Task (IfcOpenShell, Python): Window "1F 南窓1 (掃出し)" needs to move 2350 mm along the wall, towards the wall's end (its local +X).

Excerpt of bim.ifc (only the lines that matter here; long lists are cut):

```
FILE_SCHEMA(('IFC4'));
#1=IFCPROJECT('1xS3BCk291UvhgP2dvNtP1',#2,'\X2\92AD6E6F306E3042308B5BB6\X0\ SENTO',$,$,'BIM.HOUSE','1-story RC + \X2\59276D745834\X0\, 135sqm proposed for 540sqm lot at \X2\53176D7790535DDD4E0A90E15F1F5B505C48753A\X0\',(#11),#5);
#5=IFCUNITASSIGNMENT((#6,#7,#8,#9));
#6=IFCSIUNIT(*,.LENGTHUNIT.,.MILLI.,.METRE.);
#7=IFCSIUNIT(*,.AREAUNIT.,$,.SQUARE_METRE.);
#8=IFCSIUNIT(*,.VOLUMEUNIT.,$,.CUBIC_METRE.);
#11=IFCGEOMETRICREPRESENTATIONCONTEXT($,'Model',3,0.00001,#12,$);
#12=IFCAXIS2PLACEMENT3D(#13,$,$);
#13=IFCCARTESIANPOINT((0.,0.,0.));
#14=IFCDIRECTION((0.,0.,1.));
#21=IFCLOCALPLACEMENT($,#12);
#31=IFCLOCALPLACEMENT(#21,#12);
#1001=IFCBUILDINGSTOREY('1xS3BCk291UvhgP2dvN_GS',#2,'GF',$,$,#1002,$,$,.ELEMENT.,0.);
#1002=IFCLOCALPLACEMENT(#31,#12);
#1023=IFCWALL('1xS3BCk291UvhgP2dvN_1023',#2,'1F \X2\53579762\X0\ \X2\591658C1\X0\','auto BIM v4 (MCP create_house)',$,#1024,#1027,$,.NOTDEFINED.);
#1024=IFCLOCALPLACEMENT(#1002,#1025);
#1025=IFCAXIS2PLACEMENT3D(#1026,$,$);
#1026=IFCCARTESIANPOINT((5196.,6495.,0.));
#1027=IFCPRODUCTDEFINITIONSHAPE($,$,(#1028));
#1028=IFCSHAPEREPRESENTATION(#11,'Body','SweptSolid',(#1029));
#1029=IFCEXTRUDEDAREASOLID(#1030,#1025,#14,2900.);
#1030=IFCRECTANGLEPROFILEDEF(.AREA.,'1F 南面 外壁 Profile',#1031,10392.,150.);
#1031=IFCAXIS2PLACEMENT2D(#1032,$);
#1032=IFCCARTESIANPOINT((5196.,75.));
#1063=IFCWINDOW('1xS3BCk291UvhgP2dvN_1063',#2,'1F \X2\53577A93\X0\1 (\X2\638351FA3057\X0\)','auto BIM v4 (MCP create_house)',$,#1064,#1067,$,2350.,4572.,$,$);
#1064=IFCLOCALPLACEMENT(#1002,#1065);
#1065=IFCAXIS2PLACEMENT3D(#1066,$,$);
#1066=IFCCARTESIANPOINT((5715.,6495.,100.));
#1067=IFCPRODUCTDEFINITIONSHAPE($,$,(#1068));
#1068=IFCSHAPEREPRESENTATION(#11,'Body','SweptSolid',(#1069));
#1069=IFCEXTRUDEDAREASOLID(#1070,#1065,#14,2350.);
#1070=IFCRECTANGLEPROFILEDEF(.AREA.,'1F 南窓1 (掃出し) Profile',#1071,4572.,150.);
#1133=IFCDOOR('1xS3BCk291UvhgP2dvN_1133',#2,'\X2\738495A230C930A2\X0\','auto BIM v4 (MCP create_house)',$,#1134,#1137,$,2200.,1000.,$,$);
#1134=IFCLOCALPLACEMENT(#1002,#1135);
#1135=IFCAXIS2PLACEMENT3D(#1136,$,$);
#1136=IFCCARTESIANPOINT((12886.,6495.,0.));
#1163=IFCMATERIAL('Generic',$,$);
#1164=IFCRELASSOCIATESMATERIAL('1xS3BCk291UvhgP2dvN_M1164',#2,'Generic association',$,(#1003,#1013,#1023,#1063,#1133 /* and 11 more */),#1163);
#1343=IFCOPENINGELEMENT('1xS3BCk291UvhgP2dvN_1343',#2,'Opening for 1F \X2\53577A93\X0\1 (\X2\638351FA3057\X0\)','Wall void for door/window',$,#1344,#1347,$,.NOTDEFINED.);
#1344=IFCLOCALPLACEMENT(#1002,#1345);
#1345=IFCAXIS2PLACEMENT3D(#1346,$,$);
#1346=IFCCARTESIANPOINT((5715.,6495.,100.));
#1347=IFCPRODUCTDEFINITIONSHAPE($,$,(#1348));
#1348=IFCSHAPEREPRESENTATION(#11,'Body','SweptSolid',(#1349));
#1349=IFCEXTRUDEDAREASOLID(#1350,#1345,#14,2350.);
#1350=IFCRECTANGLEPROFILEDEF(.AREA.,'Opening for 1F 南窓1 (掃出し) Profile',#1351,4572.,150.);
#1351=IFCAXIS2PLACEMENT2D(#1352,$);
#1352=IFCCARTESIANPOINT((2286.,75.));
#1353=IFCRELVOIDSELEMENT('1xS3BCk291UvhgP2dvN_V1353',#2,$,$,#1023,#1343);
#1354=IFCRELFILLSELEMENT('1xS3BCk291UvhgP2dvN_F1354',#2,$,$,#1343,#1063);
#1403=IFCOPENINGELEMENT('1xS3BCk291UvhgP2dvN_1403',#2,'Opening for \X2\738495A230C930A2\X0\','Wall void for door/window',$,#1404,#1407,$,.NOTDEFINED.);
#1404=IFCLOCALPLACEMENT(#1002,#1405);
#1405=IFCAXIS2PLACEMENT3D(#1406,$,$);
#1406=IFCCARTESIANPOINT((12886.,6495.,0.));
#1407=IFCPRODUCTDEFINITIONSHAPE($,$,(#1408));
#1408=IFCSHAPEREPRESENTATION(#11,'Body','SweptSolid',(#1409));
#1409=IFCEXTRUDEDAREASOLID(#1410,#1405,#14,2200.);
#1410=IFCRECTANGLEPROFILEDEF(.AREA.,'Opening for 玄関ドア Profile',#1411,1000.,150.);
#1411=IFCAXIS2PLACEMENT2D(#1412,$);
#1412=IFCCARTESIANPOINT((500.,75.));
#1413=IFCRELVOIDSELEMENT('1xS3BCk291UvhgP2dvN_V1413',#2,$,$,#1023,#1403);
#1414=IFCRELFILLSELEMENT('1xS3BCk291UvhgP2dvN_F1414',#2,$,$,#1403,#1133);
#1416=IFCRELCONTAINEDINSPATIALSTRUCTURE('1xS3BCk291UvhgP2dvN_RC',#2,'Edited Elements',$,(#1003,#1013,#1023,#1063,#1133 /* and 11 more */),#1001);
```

```python
import ifcopenshell
import ifcopenshell.api.geometry
import ifcopenshell.util.placement
import ifcopenshell.util.unit

model = ifcopenshell.open("bim.ifc")
unit_scale = ifcopenshell.util.unit.calculate_unit_scale(model)

window = model.by_guid("1xS3BCk291UvhgP2dvN_1063")
opening = window.FillsVoids[0].RelatingOpeningElement
wall = opening.VoidsElements[0].RelatingBuildingElement

wall_matrix = ifcopenshell.util.placement.get_local_placement(wall.ObjectPlacement)
shift = wall_matrix[:3, 0] * 2.35 / unit_scale
before = ifcopenshell.util.placement.get_local_placement(window.ObjectPlacement)[:3, 3].copy()

# The window is not placed relative to its opening, so move both.
for product in (opening, window):
    matrix = ifcopenshell.util.placement.get_local_placement(product.ObjectPlacement)
    matrix[:3, 3] += shift
    ifcopenshell.api.geometry.edit_object_placement(model, product=product, matrix=matrix, is_si=False)

after = ifcopenshell.util.placement.get_local_placement(window.ObjectPlacement)[:3, 3]
print("window moved by", (after - before).round(3) + 0.0)

model.write("bim_v2.ifc")
```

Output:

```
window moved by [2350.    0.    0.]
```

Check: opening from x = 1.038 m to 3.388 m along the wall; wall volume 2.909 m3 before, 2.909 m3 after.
